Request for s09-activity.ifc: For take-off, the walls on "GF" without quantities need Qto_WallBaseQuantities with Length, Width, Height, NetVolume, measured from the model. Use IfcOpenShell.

First a look at what the model holds.

```python
import ifcopenshell
import ifcopenshell.util.element
import ifcopenshell.util.unit

model = ifcopenshell.open("s09-activity.ifc")
print(model.schema)
for unit_type in ("LENGTHUNIT", "AREAUNIT", "VOLUMEUNIT"):
    print(unit_type, ifcopenshell.util.unit.calculate_unit_scale(model, unit_type))
storey = next(s for s in model.by_type("IfcBuildingStorey") if s.Name == "GF")
walls = [e for e in ifcopenshell.util.element.get_decomposition(storey) if e.is_a("IfcWall")]
for e in sorted(walls, key=lambda e: e.id()):
    print(e.id(), e.is_a(), e.Name, list(ifcopenshell.util.element.get_psets(e, qtos_only=True)), sep=" | ")
```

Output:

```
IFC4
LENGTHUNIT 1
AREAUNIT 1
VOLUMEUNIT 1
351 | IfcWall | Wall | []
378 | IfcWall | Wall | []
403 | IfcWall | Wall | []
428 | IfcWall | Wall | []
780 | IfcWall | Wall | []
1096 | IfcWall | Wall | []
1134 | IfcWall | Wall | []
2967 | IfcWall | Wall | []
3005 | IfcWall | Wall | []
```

```python
import ifcopenshell
import ifcopenshell.api.pset
import ifcopenshell.geom
import ifcopenshell.util.element
import ifcopenshell.util.shape
import ifcopenshell.util.unit

model = ifcopenshell.open("s09-activity.ifc")
unit_scale = ifcopenshell.util.unit.calculate_unit_scale(model)
volume_scale = ifcopenshell.util.unit.calculate_unit_scale(model, "VOLUMEUNIT")
settings = ifcopenshell.geom.settings()

storey = next(s for s in model.by_type("IfcBuildingStorey") if s.Name == "GF")
walls = [e for e in ifcopenshell.util.element.get_decomposition(storey) if e.is_a("IfcWall")]

for e in sorted(walls, key=lambda e: e.id()):
    if ifcopenshell.util.element.get_psets(e, qtos_only=True, should_inherit=False):
        continue
    # Geometry comes back in metres, in the element's own axes.
    shape = ifcopenshell.geom.create_shape(settings, e)
    values = {
        "Length": ifcopenshell.util.shape.get_x(shape.geometry) / unit_scale,
        "Width": ifcopenshell.util.shape.get_y(shape.geometry) / unit_scale,
        "Height": ifcopenshell.util.shape.get_z(shape.geometry) / unit_scale,
        "NetVolume": ifcopenshell.util.shape.get_volume(shape.geometry) / volume_scale,
    }
    qto = ifcopenshell.api.pset.add_qto(model, product=e, name="Qto_WallBaseQuantities")
    ifcopenshell.api.pset.edit_qto(model, qto=qto, properties=values)
    print(e.id(), {k: round(v, 3) for k, v in values.items()})

model.write("s09-activity_updated.ifc")
```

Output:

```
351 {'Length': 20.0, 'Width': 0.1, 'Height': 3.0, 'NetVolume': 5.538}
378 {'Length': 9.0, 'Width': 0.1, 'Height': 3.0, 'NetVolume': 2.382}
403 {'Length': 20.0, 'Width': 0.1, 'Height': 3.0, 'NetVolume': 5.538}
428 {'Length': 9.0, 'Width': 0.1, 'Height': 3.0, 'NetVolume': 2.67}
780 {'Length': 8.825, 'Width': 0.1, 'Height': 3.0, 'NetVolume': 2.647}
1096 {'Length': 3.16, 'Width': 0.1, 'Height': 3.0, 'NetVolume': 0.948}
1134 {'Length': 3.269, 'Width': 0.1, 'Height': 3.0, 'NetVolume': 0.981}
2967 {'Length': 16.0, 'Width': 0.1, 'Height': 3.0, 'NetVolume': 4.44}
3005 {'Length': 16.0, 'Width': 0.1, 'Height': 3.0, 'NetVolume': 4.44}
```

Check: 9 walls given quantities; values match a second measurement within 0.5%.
